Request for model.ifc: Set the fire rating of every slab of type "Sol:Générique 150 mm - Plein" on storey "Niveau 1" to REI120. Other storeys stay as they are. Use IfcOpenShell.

First a look at what the model holds.

```python
import ifcopenshell
import ifcopenshell.util.element

model = ifcopenshell.open("model.ifc")
print(model.schema)
storey = next(s for s in model.by_type("IfcBuildingStorey") if s.Name == "Niveau 1")
slabs = [e for e in ifcopenshell.util.element.get_decomposition(storey) if e.is_a("IfcSlab")]
seen = {}
for e in slabs:
    element_type = ifcopenshell.util.element.get_type(e)
    key = (element_type.Name if element_type != e and element_type else None, ifcopenshell.util.element.get_pset(e, "Pset_SlabCommon", "FireRating"))
    seen[key] = seen.get(key, 0) + 1
for (name, value), count in sorted(seen.items(), key=str):
    print(count, "x", name, "|", value)
```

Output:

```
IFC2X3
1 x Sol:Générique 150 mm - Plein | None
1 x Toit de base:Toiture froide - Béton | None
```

```python
import ifcopenshell
import ifcopenshell.api.pset
import ifcopenshell.util.element

model = ifcopenshell.open("model.ifc")

storey = next(s for s in model.by_type("IfcBuildingStorey") if s.Name == "Niveau 1")
slabs = [e for e in ifcopenshell.util.element.get_decomposition(storey) if e.is_a("IfcSlab")]

count = 0
for e in slabs:
    element_type = ifcopenshell.util.element.get_type(e)
    if element_type in (None, e) or element_type.Name != "Sol:Générique 150 mm - Plein":
        continue
    # add_pset returns the element's existing set when there is one.
    pset = ifcopenshell.api.pset.add_pset(model, product=e, name="Pset_SlabCommon")
    ifcopenshell.api.pset.edit_pset(model, pset=pset, properties={"FireRating": "REI120"})
    count += 1

print(count, "slabs updated")

model.write("model_updated.ifc")
```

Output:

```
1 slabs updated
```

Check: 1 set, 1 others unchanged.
